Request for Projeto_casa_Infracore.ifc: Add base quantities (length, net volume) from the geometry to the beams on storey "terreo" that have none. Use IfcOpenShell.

First a look at what the model holds.

```python
import ifcopenshell
import ifcopenshell.util.element
import ifcopenshell.util.unit

model = ifcopenshell.open("Projeto_casa_Infracore.ifc")
print(model.schema)
for unit_type in ("LENGTHUNIT", "AREAUNIT", "VOLUMEUNIT"):
    print(unit_type, ifcopenshell.util.unit.calculate_unit_scale(model, unit_type))
storey = next(s for s in model.by_type("IfcBuildingStorey") if s.Name == "terreo")
beams = [e for e in ifcopenshell.util.element.get_decomposition(storey) if e.is_a("IfcBeam")]
for e in sorted(beams, key=lambda e: e.id()):
    print(e.id(), e.is_a(), e.Name, list(ifcopenshell.util.element.get_psets(e, qtos_only=True)), sep=" | ")
```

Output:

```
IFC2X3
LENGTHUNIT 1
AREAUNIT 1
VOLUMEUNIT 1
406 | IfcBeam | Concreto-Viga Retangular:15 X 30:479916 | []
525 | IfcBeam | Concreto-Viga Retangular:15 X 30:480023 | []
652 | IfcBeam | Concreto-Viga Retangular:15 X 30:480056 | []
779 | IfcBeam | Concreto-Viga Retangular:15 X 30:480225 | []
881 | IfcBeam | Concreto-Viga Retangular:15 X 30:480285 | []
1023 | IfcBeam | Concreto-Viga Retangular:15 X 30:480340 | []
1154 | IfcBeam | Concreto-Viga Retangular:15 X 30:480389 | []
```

```python
import ifcopenshell
import ifcopenshell.api.pset
import ifcopenshell.geom
import ifcopenshell.util.element
import ifcopenshell.util.shape
import ifcopenshell.util.unit

model = ifcopenshell.open("Projeto_casa_Infracore.ifc")
unit_scale = ifcopenshell.util.unit.calculate_unit_scale(model)
volume_scale = ifcopenshell.util.unit.calculate_unit_scale(model, "VOLUMEUNIT")
settings = ifcopenshell.geom.settings()

storey = next(s for s in model.by_type("IfcBuildingStorey") if s.Name == "terreo")
beams = [e for e in ifcopenshell.util.element.get_decomposition(storey) if e.is_a("IfcBeam")]

for e in sorted(beams, key=lambda e: e.id()):
    if ifcopenshell.util.element.get_psets(e, qtos_only=True, should_inherit=False):
        continue
    # Geometry comes back in metres, in the element's own axes.
    shape = ifcopenshell.geom.create_shape(settings, e)
    values = {
        "Length": ifcopenshell.util.shape.get_max_xyz(shape.geometry) / unit_scale,
        "NetVolume": ifcopenshell.util.shape.get_volume(shape.geometry) / volume_scale,
    }
    qto = ifcopenshell.api.pset.add_qto(model, product=e, name="BaseQuantities")
    ifcopenshell.api.pset.edit_qto(model, qto=qto, properties=values)
    print(e.id(), {k: round(v, 3) for k, v in values.items()})

model.write("Projeto_casa_Infracore_edited.ifc")
```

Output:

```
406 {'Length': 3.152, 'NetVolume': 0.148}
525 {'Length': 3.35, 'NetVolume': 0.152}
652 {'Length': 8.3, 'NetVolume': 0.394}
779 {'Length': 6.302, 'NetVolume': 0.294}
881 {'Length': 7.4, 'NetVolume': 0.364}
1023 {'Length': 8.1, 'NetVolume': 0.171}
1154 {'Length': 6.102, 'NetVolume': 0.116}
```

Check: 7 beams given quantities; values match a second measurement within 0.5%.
